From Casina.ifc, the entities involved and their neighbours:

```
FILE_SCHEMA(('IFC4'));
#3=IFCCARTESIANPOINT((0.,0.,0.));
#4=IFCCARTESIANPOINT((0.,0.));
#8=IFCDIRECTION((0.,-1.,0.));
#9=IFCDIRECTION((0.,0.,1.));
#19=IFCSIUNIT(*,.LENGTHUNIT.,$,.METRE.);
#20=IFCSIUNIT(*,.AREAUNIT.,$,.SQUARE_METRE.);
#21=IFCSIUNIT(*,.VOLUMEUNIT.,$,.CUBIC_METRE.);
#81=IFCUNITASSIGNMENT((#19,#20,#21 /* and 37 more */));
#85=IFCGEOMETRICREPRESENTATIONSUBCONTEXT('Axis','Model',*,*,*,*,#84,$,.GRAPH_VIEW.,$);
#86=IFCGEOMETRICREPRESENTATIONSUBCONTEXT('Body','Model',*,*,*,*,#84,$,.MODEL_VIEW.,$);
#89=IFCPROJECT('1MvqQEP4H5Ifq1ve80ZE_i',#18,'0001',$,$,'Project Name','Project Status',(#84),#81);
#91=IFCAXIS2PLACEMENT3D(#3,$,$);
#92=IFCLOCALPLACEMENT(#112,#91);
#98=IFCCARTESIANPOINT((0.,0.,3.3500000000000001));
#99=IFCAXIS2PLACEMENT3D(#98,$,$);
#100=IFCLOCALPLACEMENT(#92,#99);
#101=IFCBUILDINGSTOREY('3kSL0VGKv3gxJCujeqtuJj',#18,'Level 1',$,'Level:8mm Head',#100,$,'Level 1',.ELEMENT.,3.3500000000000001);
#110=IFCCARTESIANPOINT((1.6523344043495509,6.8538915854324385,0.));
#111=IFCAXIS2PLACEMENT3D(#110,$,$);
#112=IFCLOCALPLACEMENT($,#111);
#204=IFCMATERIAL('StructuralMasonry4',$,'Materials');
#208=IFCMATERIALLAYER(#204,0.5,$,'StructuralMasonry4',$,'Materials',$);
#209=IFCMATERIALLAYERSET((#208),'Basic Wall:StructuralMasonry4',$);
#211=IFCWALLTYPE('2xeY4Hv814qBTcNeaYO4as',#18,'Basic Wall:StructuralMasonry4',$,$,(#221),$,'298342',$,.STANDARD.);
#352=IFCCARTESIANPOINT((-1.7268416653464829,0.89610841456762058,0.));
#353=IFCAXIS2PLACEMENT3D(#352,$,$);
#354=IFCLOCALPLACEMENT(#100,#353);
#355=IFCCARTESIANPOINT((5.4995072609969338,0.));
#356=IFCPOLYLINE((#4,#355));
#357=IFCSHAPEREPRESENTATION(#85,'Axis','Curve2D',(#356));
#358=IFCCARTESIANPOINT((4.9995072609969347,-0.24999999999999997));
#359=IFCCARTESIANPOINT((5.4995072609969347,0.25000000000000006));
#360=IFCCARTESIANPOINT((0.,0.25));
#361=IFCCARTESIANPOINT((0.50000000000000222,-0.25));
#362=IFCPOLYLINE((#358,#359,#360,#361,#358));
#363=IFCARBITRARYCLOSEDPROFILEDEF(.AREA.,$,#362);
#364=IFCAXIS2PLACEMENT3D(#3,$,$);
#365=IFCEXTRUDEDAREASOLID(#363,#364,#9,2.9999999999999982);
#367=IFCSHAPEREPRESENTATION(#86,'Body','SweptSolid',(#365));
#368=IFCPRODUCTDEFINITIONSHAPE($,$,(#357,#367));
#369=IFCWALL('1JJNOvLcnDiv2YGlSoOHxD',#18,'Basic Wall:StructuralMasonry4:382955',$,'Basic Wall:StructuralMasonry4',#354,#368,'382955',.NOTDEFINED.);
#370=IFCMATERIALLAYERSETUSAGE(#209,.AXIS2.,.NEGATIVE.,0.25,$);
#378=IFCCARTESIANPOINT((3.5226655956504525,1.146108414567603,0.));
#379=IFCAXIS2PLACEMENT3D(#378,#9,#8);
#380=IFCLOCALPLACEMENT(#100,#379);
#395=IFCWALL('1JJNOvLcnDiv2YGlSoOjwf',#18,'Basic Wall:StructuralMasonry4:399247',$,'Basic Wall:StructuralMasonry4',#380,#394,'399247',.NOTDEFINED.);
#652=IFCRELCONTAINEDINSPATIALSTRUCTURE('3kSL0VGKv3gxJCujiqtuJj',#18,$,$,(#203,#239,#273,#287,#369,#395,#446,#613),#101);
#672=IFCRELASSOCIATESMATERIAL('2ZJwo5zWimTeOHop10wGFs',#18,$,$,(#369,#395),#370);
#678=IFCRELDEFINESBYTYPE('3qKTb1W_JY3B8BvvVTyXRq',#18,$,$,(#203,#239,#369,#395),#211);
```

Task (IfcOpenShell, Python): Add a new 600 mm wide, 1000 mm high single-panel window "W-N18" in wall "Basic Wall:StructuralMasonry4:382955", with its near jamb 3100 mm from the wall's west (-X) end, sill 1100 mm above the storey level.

```python
import numpy as np
import ifcopenshell
import ifcopenshell.api.feature
import ifcopenshell.api.geometry
import ifcopenshell.api.root
import ifcopenshell.api.spatial
import ifcopenshell.geom
import ifcopenshell.util.element
import ifcopenshell.util.placement
import ifcopenshell.util.representation
import ifcopenshell.util.shape
import ifcopenshell.util.unit

model = ifcopenshell.open("Casina.ifc")
unit_scale = ifcopenshell.util.unit.calculate_unit_scale(model)
settings = ifcopenshell.geom.settings()


def volume(element):
    """Net volume in cubic metres, openings subtracted."""
    shape = ifcopenshell.geom.create_shape(settings, element)
    return ifcopenshell.util.shape.get_volume(shape.geometry)


wall = model.by_guid("1JJNOvLcnDiv2YGlSoOHxD")
storey = ifcopenshell.util.element.get_container(wall, ifc_class="IfcBuildingStorey")
context = ifcopenshell.util.representation.get_context(model, "Model", "Body", "MODEL_VIEW")
before = volume(wall)

width, height, from_end, sill = 0.6, 1, 3.1, 1.1  # metres

# The wall runs along its own X axis, and the end named is its -X end.
wall_shape = ifcopenshell.geom.create_shape(settings, wall)
x, y, z = ifcopenshell.util.shape.get_vertices(wall_shape.geometry).T
start = x.min() + from_end
face, thickness = float(y.min()), float(y.max() - y.min())
wall_matrix = ifcopenshell.util.placement.get_local_placement(wall.ObjectPlacement)
level = ifcopenshell.util.placement.get_local_placement(storey.ObjectPlacement)[2, 3]


def in_wall(x, y):
    """Placement at x, y metres in the wall's axes, at sill height."""
    matrix = wall_matrix.copy()
    matrix[:, 3] = wall_matrix @ np.array([x / unit_scale, y / unit_scale, 0.0, 1.0])
    matrix[2, 3] = level + sill / unit_scale
    return matrix


# Opening: a box that overshoots both wall faces by 50 mm.
opening = ifcopenshell.api.root.create_entity(model, ifc_class="IfcOpeningElement", predefined_type="OPENING")
box = ifcopenshell.api.geometry.add_wall_representation(
    model, context=context, length=width, height=height, thickness=thickness + 0.1
)
ifcopenshell.api.geometry.assign_representation(model, product=opening, representation=box)
ifcopenshell.api.geometry.edit_object_placement(model, product=opening, matrix=in_wall(start, face - 0.05), is_si=False)
ifcopenshell.api.feature.add_feature(model, feature=opening, element=wall)

window = ifcopenshell.api.root.create_entity(model, ifc_class="IfcWindow", name="W-N18", predefined_type="WINDOW")
window.OverallWidth, window.OverallHeight = width / unit_scale, height / unit_scale
window.PartitioningType = "SINGLE_PANEL"
body = ifcopenshell.api.geometry.add_window_representation(
    model,
    context=context,
    overall_width=window.OverallWidth,
    overall_height=window.OverallHeight,
    partition_type="SINGLE_PANEL",
)
ifcopenshell.api.geometry.assign_representation(model, product=window, representation=body)
ifcopenshell.api.spatial.assign_container(model, products=[window], relating_structure=storey)
ifcopenshell.api.feature.add_filling(model, opening=opening, element=window)

# Centre the window in the wall's thickness.
ifcopenshell.api.geometry.edit_object_placement(model, product=window, matrix=in_wall(start, face), is_si=False)
window_shape = ifcopenshell.geom.create_shape(settings, window)
depth = ifcopenshell.util.shape.get_vertices(window_shape.geometry)[:, 1]
offset = face + thickness / 2 - (depth.min() + depth.max()) / 2
ifcopenshell.api.geometry.edit_object_placement(model, product=window, matrix=in_wall(start, offset), is_si=False)

after = volume(wall)

print(f"wall volume {before:.3f} -> {after:.3f} m3")

model.write("Casina_updated.ifc")
```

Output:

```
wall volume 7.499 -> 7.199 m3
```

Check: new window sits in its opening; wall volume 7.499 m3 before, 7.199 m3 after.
